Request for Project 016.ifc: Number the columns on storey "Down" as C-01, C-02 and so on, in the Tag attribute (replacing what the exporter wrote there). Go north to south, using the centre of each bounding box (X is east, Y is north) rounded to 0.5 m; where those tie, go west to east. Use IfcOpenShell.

First a look at what the model holds.

```python
import ifcopenshell
import ifcopenshell.util.element
import ifcopenshell.util.placement

model = ifcopenshell.open("Project 016.ifc")
print(model.schema)
storey = next(s for s in model.by_type("IfcBuildingStorey") if s.Name == "Down")
columns = [e for e in ifcopenshell.util.element.get_decomposition(storey) if e.is_a("IfcColumn")]
for e in sorted(columns, key=lambda e: e.id()):
    origin = ifcopenshell.util.placement.get_local_placement(e.ObjectPlacement)[:3, 3]
    print(e.id(), e.Tag, e.Name, origin.round(2) + 0.0, sep=" | ")
```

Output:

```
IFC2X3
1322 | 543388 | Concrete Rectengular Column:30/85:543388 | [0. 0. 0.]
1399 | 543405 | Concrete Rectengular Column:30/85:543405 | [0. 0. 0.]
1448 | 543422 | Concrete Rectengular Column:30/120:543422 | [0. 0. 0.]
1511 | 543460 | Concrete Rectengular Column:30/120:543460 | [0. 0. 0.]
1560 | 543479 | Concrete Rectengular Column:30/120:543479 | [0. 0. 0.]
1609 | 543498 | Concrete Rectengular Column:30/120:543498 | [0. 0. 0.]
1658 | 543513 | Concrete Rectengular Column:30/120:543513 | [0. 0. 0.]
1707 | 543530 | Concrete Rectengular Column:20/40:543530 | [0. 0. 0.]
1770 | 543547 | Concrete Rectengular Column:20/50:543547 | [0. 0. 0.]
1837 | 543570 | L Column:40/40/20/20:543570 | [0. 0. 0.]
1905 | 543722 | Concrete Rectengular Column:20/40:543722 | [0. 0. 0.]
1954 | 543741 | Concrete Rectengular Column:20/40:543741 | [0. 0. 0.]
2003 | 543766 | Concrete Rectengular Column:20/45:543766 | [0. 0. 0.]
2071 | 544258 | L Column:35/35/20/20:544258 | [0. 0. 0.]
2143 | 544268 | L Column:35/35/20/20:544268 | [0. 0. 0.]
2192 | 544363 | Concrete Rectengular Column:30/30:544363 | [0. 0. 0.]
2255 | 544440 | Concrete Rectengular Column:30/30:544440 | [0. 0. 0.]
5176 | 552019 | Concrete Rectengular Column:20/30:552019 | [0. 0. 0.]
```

```python
import ifcopenshell
import ifcopenshell.geom
import ifcopenshell.util.element
import ifcopenshell.util.shape

model = ifcopenshell.open("Project 016.ifc")
settings = ifcopenshell.geom.settings()
settings.set("use-world-coords", True)


def centre(element):
    shape = ifcopenshell.geom.create_shape(settings, element)
    return ifcopenshell.util.shape.get_bbox_centroid(shape.geometry)


storey = next(s for s in model.by_type("IfcBuildingStorey") if s.Name == "Down")
columns = [e for e in ifcopenshell.util.element.get_decomposition(storey) if e.is_a("IfcColumn")]

# Insertion points can sit at a corner or the storey origin, so sort by the geometry (in metres).
centres = {e: centre(e) for e in columns}
columns.sort(key=lambda e: (-round(centres[e][1] / 0.5), centres[e][0]))

for i, e in enumerate(columns, start=1):
    number = f"C-{i:02d}"
    e.Tag = number
    print(e.id(), number)

model.write("Project 016_edited.ifc")
```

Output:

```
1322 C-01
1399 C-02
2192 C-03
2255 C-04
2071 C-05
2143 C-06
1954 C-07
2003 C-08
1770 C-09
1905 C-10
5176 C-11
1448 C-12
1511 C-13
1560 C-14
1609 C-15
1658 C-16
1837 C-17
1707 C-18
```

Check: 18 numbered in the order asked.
